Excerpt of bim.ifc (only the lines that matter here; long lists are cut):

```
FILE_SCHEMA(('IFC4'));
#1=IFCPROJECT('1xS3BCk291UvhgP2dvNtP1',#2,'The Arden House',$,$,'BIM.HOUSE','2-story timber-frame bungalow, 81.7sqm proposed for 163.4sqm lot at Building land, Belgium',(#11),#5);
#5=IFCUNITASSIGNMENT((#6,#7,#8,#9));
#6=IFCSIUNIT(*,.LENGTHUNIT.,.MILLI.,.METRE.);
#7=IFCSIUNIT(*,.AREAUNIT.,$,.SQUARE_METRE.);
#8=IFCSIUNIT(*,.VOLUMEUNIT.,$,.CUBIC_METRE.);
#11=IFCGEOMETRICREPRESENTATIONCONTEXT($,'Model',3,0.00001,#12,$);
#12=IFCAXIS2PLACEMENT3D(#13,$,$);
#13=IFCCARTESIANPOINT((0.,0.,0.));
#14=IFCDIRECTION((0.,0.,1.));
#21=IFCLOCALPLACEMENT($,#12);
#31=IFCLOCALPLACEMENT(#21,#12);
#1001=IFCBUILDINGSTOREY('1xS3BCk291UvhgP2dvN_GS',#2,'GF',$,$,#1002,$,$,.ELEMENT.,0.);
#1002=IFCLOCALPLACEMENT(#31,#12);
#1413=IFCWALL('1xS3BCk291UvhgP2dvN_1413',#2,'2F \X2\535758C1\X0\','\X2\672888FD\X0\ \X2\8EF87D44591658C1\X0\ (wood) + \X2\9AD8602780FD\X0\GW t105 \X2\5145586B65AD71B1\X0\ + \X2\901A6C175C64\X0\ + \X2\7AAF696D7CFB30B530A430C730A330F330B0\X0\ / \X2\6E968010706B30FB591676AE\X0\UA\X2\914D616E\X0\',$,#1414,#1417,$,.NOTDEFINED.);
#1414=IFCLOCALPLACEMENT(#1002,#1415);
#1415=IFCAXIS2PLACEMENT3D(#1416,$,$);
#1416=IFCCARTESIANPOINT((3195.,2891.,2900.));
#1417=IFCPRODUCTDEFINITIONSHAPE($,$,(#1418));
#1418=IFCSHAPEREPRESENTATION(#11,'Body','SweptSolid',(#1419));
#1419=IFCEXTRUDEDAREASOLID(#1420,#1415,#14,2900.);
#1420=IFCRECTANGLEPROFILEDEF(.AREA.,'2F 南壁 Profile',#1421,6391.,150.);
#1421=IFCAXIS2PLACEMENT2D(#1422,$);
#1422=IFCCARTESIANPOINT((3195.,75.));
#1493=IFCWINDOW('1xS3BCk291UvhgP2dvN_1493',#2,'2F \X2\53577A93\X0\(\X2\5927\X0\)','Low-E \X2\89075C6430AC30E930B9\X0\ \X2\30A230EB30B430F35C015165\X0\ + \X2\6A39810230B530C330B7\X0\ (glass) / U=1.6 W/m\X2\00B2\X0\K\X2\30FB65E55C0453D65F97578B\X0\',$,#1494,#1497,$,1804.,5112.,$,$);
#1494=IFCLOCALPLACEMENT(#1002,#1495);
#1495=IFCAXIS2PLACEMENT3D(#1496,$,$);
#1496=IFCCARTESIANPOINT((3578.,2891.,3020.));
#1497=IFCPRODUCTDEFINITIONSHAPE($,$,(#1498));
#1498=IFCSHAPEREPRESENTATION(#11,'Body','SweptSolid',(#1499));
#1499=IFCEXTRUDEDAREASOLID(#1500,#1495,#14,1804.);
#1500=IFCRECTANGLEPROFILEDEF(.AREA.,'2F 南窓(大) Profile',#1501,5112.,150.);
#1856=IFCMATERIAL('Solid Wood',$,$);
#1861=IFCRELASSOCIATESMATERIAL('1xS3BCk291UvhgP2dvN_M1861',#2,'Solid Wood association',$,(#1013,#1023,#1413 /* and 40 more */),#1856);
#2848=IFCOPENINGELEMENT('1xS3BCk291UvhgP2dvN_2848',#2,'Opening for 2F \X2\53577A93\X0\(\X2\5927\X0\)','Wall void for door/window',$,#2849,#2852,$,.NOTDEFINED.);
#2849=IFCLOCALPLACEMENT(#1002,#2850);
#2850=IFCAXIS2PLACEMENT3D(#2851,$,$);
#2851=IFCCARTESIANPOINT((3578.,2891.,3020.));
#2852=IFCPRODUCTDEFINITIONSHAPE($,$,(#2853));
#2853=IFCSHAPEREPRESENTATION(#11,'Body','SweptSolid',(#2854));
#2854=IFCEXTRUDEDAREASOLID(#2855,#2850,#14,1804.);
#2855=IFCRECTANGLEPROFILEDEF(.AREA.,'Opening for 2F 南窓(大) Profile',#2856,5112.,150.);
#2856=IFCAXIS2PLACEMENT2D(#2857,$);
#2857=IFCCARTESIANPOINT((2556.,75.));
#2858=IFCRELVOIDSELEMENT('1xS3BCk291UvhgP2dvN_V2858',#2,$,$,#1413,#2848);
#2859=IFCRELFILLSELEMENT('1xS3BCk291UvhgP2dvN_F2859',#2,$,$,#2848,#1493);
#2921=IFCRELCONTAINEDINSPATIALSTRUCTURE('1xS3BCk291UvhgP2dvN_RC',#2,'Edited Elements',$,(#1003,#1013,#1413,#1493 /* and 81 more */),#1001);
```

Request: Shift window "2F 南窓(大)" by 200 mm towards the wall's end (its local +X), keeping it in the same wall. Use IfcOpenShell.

```python
import ifcopenshell
import ifcopenshell.api.geometry
import ifcopenshell.util.placement

model = ifcopenshell.open("bim.ifc")

window = model.by_guid("1xS3BCk291UvhgP2dvN_1493")
opening = window.FillsVoids[0].RelatingOpeningElement
wall = opening.VoidsElements[0].RelatingBuildingElement

wall_matrix = ifcopenshell.util.placement.get_local_placement(wall.ObjectPlacement)
shift = wall_matrix[:3, 0] * 200.0
before = ifcopenshell.util.placement.get_local_placement(window.ObjectPlacement)[:3, 3].copy()

# The window is not placed relative to its opening, so move both.
for product in (opening, window):
    matrix = ifcopenshell.util.placement.get_local_placement(product.ObjectPlacement)
    matrix[:3, 3] += shift
    ifcopenshell.api.geometry.edit_object_placement(model, product=product, matrix=matrix, is_si=False)

after = ifcopenshell.util.placement.get_local_placement(window.ObjectPlacement)[:3, 3]
print("window moved by", (after - before).round(3) + 0.0)

model.write("bim_updated.ifc")
```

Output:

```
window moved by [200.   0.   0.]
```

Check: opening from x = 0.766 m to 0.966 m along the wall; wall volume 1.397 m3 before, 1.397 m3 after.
